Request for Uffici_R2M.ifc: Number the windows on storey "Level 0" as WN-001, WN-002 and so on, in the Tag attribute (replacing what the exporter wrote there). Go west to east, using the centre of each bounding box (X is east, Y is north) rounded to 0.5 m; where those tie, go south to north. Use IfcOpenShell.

First a look at what the model holds.

```python
import ifcopenshell
import ifcopenshell.util.element
import ifcopenshell.util.placement

model = ifcopenshell.open("Uffici_R2M.ifc")
print(model.schema)
storey = next(s for s in model.by_type("IfcBuildingStorey") if s.Name == "Level 0")
windows = [e for e in ifcopenshell.util.element.get_decomposition(storey) if e.is_a("IfcWindow")]
for e in sorted(windows, key=lambda e: e.id()):
    origin = ifcopenshell.util.placement.get_local_placement(e.ObjectPlacement)[:3, 3]
    print(e.id(), e.Tag, e.Name, origin.round(2) + 0.0, sep=" | ")
```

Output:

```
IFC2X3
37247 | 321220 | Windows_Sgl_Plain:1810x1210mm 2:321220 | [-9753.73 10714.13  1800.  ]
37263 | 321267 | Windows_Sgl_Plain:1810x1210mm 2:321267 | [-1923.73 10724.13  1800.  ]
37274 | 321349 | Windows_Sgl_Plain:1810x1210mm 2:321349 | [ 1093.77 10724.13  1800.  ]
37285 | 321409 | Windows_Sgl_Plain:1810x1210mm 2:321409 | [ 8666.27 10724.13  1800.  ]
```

```python
import ifcopenshell
import ifcopenshell.geom
import ifcopenshell.util.element
import ifcopenshell.util.shape

model = ifcopenshell.open("Uffici_R2M.ifc")
settings = ifcopenshell.geom.settings()
settings.set("use-world-coords", True)


def centre(element):
    shape = ifcopenshell.geom.create_shape(settings, element)
    return ifcopenshell.util.shape.get_bbox_centroid(shape.geometry)


storey = next(s for s in model.by_type("IfcBuildingStorey") if s.Name == "Level 0")
windows = [e for e in ifcopenshell.util.element.get_decomposition(storey) if e.is_a("IfcWindow")]

# Insertion points can sit at a corner or the storey origin, so sort by the geometry (in metres).
centres = {e: centre(e) for e in windows}
windows.sort(key=lambda e: (round(centres[e][0] / 0.5), centres[e][1]))

for i, e in enumerate(windows, start=1):
    number = f"WN-0{i:02d}"
    e.Tag = number
    print(e.id(), number)

model.write("Uffici_R2M_edited.ifc")
```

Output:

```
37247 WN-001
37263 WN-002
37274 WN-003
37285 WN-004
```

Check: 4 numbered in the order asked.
